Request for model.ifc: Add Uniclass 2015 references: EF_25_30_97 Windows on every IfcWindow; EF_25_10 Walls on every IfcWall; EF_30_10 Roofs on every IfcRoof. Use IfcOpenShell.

First a look at what the model holds.

```python
import ifcopenshell

model = ifcopenshell.open("model.ifc")
print(model.schema)
print("classifications:", [c.Name for c in model.by_type("IfcClassification")])
for ifc_class in ("IfcDoor", "IfcRoof", "IfcStair", "IfcWall", "IfcWindow"):
    print(ifc_class, len(model.by_type(ifc_class)))
```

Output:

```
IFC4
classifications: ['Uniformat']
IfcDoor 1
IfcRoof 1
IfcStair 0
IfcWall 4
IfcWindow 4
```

```python
import ifcopenshell
import ifcopenshell.api.classification

model = ifcopenshell.open("model.ifc")

system = ifcopenshell.api.classification.add_classification(model, classification="Uniclass 2015")

codes = {
    "IfcWindow": ("EF_25_30_97", "Windows"),
    "IfcWall": ("EF_25_10", "Walls"),
    "IfcRoof": ("EF_30_10", "Roofs"),
}
for ifc_class, (code, name) in codes.items():
    products = model.by_type(ifc_class)
    ifcopenshell.api.classification.add_reference(
        model, products=products, classification=system, identification=code, name=name
    )
    print(code, len(products))

model.write("model_v2.ifc")
```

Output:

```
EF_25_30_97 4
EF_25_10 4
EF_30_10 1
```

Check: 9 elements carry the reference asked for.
